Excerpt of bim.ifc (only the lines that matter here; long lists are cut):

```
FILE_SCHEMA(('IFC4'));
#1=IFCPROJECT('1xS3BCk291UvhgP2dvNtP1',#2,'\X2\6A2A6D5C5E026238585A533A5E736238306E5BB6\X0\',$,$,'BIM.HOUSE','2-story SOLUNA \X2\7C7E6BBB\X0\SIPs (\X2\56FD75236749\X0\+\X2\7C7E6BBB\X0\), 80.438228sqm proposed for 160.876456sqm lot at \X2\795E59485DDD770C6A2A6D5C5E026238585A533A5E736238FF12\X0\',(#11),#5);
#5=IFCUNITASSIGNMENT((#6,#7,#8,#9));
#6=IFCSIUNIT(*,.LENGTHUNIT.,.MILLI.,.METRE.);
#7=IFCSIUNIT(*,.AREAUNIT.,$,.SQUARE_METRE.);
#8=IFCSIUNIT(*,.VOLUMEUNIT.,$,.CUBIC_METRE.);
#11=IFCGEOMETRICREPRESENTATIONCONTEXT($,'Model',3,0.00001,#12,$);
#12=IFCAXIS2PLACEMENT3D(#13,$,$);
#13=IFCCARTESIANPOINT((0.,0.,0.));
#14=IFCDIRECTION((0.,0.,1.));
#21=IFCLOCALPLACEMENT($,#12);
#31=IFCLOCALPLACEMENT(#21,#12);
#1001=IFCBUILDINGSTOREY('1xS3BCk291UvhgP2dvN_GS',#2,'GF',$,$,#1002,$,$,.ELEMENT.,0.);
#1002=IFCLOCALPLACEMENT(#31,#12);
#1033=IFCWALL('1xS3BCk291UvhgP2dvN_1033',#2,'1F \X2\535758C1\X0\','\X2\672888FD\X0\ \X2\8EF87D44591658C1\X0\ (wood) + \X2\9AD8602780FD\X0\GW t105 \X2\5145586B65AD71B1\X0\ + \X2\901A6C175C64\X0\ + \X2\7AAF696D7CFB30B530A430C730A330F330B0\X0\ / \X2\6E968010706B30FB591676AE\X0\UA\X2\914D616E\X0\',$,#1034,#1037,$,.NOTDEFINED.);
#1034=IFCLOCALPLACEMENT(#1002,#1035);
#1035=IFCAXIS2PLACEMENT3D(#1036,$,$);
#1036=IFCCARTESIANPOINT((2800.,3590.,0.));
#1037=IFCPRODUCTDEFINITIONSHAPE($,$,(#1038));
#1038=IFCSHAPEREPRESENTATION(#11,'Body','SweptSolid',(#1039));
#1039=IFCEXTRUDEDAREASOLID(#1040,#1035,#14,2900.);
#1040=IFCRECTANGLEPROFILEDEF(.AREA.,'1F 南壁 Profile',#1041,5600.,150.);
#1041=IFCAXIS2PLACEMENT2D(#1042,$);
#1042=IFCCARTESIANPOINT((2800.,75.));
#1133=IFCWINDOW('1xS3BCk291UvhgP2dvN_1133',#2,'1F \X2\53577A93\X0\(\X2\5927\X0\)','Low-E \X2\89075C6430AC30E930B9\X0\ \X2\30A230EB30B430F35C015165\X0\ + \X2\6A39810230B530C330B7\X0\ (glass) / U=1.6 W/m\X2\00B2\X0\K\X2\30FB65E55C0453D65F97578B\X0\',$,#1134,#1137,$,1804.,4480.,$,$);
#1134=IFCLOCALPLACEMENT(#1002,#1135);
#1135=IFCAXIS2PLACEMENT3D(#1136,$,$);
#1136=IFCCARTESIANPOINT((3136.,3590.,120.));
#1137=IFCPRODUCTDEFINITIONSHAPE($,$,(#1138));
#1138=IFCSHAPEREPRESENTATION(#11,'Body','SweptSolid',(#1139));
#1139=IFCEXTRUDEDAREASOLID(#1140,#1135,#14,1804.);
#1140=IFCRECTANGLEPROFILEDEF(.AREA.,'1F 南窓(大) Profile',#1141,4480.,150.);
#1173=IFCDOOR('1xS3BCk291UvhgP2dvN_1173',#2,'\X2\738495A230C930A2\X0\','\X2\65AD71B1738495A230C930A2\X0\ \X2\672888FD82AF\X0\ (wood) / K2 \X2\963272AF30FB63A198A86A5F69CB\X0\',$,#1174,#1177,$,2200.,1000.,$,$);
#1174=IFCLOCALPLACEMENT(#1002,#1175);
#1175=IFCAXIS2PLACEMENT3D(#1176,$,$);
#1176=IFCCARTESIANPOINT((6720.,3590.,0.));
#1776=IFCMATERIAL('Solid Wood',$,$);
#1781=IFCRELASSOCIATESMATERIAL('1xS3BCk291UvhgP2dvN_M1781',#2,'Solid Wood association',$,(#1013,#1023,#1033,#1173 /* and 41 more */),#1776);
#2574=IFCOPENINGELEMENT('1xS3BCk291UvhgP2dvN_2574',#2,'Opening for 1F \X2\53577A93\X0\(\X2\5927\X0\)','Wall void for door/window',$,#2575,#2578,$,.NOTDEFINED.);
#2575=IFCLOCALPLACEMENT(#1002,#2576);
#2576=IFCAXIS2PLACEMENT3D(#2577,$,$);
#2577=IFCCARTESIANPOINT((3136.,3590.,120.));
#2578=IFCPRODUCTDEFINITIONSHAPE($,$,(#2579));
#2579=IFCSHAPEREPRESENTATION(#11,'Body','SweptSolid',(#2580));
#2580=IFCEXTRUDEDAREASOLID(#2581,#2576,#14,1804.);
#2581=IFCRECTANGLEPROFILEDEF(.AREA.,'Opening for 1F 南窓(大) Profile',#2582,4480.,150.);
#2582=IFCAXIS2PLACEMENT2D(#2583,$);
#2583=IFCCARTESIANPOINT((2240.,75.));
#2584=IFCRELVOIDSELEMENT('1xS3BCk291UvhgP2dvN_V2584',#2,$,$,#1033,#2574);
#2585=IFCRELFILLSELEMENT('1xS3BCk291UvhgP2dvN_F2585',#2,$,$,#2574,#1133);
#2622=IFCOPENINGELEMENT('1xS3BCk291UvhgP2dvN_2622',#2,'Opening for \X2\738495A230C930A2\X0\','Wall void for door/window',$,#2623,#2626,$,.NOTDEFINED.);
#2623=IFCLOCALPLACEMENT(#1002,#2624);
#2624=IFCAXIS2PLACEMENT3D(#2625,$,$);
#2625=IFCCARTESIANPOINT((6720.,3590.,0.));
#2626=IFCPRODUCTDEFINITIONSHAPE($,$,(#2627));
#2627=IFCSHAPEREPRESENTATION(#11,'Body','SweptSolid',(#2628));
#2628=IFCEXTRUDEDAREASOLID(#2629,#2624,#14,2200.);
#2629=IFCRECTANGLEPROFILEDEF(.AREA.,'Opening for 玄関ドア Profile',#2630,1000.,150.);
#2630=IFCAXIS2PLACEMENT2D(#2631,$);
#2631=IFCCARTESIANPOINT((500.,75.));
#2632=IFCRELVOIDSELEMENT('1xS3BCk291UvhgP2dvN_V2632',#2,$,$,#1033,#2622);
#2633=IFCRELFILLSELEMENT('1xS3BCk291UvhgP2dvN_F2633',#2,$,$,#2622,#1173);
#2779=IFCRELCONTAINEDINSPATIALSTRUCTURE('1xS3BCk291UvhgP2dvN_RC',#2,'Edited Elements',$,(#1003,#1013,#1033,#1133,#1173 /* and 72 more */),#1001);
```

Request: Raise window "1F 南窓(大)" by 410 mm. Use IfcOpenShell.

```python
import numpy as np
import ifcopenshell
import ifcopenshell.api.geometry
import ifcopenshell.util.placement
import ifcopenshell.util.unit

model = ifcopenshell.open("bim.ifc")
unit_scale = ifcopenshell.util.unit.calculate_unit_scale(model)

window = model.by_guid("1xS3BCk291UvhgP2dvN_1133")
opening = window.FillsVoids[0].RelatingOpeningElement
dz = 410.0

shift = np.array([0.0, 0.0, dz])
# The window is not placed relative to its opening, so move both.
for product in (opening, window):
    matrix = ifcopenshell.util.placement.get_local_placement(product.ObjectPlacement)
    matrix[:3, 3] += shift
    ifcopenshell.api.geometry.edit_object_placement(model, product=product, matrix=matrix, is_si=False)

print(f"moved by {dz * unit_scale:+.3f} m")

model.write("bim_rev.ifc")
```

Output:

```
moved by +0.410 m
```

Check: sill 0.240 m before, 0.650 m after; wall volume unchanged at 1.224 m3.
